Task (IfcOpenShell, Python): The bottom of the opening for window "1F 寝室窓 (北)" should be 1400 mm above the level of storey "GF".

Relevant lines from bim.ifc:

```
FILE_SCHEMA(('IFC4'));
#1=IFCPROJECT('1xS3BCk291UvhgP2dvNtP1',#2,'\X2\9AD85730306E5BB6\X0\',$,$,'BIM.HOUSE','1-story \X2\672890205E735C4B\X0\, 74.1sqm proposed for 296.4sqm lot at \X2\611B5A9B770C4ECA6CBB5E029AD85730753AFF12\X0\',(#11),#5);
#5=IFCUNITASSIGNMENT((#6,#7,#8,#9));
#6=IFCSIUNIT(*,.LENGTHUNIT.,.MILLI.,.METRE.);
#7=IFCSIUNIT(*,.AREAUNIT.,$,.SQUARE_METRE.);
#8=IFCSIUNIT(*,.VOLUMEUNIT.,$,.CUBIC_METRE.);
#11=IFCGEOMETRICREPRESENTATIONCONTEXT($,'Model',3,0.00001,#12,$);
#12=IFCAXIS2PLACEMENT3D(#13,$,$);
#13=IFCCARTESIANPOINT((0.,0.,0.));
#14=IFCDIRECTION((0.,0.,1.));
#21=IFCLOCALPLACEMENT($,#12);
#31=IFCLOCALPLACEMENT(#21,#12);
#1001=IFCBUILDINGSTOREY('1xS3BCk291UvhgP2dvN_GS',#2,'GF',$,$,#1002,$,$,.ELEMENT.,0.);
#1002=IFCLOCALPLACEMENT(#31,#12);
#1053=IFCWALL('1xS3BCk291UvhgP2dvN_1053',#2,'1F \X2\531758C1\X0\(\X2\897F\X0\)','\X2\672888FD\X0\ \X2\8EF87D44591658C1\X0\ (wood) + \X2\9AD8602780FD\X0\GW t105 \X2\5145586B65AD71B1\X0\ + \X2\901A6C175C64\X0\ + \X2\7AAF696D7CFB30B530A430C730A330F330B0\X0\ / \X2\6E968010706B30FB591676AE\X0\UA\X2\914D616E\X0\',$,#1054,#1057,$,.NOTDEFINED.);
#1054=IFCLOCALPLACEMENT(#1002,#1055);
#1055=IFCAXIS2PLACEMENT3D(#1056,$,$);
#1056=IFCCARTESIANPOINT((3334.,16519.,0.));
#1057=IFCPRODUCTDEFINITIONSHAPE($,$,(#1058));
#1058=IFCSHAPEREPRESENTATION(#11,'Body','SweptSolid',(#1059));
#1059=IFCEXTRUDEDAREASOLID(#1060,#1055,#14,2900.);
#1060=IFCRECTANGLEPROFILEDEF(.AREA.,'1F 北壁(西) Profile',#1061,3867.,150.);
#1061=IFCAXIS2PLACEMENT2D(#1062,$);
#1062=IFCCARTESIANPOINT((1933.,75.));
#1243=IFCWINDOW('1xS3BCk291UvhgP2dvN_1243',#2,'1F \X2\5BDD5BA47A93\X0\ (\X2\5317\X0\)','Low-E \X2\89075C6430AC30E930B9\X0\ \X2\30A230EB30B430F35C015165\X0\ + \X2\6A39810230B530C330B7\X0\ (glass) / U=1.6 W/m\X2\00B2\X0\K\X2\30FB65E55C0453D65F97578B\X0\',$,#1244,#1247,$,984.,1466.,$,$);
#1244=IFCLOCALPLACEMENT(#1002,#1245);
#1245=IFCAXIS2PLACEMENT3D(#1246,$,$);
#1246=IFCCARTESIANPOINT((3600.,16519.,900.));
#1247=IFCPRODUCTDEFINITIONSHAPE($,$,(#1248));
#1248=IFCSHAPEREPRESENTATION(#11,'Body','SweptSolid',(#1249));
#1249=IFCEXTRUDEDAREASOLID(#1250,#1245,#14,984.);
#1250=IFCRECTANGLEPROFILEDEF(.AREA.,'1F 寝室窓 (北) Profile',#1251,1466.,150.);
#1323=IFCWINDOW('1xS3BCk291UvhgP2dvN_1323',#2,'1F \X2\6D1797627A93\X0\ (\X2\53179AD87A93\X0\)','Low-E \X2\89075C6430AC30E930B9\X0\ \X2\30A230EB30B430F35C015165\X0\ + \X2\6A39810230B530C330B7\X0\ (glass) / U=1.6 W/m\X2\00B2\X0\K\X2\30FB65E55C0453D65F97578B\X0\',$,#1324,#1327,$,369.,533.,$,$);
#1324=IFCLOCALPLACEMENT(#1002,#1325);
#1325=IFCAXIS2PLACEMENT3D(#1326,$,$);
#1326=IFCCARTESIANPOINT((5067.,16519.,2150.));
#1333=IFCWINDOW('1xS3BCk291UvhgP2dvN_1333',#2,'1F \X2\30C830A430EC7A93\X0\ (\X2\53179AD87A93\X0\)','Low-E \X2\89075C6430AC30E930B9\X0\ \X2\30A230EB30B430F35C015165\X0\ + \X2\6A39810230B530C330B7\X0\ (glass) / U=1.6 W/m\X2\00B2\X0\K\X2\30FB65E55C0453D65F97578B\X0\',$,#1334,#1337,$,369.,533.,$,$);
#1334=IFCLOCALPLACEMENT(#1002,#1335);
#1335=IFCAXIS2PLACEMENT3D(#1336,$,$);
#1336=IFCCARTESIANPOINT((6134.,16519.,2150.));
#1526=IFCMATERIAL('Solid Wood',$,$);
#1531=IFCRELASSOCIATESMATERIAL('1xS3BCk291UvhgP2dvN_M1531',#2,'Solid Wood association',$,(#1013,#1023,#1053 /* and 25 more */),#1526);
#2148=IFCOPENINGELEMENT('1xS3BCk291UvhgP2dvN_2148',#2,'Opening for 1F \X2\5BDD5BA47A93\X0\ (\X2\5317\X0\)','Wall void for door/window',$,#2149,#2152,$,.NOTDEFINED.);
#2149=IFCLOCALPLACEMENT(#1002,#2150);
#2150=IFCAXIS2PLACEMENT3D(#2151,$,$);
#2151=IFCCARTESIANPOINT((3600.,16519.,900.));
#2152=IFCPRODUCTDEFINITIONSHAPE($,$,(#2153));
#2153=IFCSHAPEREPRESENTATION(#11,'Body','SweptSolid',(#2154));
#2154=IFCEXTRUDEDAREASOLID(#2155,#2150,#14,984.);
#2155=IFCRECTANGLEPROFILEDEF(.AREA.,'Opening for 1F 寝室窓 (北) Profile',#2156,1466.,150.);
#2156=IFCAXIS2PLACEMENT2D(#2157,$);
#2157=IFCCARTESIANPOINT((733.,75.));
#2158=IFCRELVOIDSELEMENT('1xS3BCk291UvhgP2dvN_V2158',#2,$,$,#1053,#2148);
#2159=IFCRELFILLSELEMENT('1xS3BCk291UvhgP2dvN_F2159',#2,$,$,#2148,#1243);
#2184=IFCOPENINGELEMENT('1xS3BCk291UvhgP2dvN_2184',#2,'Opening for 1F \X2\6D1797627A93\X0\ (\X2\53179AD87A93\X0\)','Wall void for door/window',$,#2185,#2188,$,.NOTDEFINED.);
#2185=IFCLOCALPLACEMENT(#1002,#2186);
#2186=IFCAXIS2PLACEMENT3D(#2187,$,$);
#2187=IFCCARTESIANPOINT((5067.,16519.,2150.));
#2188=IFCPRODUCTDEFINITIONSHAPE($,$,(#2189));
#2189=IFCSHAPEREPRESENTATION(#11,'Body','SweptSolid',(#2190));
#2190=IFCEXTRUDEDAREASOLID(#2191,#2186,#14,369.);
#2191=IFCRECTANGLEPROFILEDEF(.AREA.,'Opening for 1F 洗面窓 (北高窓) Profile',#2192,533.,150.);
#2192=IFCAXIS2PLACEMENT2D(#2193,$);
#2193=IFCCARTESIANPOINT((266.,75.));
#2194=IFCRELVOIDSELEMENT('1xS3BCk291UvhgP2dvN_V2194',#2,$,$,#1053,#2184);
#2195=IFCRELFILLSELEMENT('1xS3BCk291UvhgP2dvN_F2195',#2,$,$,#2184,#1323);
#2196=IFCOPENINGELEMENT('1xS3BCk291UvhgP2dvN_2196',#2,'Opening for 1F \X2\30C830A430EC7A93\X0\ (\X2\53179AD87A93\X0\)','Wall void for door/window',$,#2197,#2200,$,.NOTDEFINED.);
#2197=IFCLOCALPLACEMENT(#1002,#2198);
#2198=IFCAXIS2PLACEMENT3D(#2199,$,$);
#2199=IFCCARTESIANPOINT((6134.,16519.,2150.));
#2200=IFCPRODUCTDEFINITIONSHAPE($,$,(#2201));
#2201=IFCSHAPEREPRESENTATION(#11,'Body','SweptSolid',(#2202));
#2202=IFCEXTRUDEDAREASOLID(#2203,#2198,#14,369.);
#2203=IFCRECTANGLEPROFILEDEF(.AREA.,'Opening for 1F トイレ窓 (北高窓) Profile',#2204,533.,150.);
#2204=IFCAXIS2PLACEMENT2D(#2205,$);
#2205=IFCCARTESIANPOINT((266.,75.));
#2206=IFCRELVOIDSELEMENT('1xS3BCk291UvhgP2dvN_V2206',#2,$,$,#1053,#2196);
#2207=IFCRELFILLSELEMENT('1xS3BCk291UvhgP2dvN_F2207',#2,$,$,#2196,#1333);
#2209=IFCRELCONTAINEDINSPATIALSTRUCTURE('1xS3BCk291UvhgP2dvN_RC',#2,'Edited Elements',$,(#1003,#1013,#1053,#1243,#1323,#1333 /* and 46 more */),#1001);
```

```python
import numpy as np
import ifcopenshell
import ifcopenshell.api.geometry
import ifcopenshell.geom
import ifcopenshell.util.element
import ifcopenshell.util.placement
import ifcopenshell.util.shape
import ifcopenshell.util.unit

model = ifcopenshell.open("bim.ifc")
unit_scale = ifcopenshell.util.unit.calculate_unit_scale(model)

window = model.by_id(1243)
opening = window.FillsVoids[0].RelatingOpeningElement
storey = ifcopenshell.util.element.get_container(window, ifc_class="IfcBuildingStorey")
level = ifcopenshell.util.placement.get_local_placement(storey.ObjectPlacement)[2, 3]

# The opening's origin need not be at the sill, so measure its lowest point.
shape = ifcopenshell.geom.create_shape(ifcopenshell.geom.settings(), opening)
bottom = ifcopenshell.util.shape.get_shape_bottom_elevation(shape, shape.geometry) / unit_scale
dz = level + 1.4 / unit_scale - bottom

shift = np.array([0.0, 0.0, dz])
# The window is not placed relative to its opening, so move both.
for product in (opening, window):
    matrix = ifcopenshell.util.placement.get_local_placement(product.ObjectPlacement)
    matrix[:3, 3] += shift
    ifcopenshell.api.geometry.edit_object_placement(model, product=product, matrix=matrix, is_si=False)

print(f"moved by {dz * unit_scale:+.3f} m")

model.write("bim_rev.ifc")
```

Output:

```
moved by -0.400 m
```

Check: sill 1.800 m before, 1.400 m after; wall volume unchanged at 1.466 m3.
